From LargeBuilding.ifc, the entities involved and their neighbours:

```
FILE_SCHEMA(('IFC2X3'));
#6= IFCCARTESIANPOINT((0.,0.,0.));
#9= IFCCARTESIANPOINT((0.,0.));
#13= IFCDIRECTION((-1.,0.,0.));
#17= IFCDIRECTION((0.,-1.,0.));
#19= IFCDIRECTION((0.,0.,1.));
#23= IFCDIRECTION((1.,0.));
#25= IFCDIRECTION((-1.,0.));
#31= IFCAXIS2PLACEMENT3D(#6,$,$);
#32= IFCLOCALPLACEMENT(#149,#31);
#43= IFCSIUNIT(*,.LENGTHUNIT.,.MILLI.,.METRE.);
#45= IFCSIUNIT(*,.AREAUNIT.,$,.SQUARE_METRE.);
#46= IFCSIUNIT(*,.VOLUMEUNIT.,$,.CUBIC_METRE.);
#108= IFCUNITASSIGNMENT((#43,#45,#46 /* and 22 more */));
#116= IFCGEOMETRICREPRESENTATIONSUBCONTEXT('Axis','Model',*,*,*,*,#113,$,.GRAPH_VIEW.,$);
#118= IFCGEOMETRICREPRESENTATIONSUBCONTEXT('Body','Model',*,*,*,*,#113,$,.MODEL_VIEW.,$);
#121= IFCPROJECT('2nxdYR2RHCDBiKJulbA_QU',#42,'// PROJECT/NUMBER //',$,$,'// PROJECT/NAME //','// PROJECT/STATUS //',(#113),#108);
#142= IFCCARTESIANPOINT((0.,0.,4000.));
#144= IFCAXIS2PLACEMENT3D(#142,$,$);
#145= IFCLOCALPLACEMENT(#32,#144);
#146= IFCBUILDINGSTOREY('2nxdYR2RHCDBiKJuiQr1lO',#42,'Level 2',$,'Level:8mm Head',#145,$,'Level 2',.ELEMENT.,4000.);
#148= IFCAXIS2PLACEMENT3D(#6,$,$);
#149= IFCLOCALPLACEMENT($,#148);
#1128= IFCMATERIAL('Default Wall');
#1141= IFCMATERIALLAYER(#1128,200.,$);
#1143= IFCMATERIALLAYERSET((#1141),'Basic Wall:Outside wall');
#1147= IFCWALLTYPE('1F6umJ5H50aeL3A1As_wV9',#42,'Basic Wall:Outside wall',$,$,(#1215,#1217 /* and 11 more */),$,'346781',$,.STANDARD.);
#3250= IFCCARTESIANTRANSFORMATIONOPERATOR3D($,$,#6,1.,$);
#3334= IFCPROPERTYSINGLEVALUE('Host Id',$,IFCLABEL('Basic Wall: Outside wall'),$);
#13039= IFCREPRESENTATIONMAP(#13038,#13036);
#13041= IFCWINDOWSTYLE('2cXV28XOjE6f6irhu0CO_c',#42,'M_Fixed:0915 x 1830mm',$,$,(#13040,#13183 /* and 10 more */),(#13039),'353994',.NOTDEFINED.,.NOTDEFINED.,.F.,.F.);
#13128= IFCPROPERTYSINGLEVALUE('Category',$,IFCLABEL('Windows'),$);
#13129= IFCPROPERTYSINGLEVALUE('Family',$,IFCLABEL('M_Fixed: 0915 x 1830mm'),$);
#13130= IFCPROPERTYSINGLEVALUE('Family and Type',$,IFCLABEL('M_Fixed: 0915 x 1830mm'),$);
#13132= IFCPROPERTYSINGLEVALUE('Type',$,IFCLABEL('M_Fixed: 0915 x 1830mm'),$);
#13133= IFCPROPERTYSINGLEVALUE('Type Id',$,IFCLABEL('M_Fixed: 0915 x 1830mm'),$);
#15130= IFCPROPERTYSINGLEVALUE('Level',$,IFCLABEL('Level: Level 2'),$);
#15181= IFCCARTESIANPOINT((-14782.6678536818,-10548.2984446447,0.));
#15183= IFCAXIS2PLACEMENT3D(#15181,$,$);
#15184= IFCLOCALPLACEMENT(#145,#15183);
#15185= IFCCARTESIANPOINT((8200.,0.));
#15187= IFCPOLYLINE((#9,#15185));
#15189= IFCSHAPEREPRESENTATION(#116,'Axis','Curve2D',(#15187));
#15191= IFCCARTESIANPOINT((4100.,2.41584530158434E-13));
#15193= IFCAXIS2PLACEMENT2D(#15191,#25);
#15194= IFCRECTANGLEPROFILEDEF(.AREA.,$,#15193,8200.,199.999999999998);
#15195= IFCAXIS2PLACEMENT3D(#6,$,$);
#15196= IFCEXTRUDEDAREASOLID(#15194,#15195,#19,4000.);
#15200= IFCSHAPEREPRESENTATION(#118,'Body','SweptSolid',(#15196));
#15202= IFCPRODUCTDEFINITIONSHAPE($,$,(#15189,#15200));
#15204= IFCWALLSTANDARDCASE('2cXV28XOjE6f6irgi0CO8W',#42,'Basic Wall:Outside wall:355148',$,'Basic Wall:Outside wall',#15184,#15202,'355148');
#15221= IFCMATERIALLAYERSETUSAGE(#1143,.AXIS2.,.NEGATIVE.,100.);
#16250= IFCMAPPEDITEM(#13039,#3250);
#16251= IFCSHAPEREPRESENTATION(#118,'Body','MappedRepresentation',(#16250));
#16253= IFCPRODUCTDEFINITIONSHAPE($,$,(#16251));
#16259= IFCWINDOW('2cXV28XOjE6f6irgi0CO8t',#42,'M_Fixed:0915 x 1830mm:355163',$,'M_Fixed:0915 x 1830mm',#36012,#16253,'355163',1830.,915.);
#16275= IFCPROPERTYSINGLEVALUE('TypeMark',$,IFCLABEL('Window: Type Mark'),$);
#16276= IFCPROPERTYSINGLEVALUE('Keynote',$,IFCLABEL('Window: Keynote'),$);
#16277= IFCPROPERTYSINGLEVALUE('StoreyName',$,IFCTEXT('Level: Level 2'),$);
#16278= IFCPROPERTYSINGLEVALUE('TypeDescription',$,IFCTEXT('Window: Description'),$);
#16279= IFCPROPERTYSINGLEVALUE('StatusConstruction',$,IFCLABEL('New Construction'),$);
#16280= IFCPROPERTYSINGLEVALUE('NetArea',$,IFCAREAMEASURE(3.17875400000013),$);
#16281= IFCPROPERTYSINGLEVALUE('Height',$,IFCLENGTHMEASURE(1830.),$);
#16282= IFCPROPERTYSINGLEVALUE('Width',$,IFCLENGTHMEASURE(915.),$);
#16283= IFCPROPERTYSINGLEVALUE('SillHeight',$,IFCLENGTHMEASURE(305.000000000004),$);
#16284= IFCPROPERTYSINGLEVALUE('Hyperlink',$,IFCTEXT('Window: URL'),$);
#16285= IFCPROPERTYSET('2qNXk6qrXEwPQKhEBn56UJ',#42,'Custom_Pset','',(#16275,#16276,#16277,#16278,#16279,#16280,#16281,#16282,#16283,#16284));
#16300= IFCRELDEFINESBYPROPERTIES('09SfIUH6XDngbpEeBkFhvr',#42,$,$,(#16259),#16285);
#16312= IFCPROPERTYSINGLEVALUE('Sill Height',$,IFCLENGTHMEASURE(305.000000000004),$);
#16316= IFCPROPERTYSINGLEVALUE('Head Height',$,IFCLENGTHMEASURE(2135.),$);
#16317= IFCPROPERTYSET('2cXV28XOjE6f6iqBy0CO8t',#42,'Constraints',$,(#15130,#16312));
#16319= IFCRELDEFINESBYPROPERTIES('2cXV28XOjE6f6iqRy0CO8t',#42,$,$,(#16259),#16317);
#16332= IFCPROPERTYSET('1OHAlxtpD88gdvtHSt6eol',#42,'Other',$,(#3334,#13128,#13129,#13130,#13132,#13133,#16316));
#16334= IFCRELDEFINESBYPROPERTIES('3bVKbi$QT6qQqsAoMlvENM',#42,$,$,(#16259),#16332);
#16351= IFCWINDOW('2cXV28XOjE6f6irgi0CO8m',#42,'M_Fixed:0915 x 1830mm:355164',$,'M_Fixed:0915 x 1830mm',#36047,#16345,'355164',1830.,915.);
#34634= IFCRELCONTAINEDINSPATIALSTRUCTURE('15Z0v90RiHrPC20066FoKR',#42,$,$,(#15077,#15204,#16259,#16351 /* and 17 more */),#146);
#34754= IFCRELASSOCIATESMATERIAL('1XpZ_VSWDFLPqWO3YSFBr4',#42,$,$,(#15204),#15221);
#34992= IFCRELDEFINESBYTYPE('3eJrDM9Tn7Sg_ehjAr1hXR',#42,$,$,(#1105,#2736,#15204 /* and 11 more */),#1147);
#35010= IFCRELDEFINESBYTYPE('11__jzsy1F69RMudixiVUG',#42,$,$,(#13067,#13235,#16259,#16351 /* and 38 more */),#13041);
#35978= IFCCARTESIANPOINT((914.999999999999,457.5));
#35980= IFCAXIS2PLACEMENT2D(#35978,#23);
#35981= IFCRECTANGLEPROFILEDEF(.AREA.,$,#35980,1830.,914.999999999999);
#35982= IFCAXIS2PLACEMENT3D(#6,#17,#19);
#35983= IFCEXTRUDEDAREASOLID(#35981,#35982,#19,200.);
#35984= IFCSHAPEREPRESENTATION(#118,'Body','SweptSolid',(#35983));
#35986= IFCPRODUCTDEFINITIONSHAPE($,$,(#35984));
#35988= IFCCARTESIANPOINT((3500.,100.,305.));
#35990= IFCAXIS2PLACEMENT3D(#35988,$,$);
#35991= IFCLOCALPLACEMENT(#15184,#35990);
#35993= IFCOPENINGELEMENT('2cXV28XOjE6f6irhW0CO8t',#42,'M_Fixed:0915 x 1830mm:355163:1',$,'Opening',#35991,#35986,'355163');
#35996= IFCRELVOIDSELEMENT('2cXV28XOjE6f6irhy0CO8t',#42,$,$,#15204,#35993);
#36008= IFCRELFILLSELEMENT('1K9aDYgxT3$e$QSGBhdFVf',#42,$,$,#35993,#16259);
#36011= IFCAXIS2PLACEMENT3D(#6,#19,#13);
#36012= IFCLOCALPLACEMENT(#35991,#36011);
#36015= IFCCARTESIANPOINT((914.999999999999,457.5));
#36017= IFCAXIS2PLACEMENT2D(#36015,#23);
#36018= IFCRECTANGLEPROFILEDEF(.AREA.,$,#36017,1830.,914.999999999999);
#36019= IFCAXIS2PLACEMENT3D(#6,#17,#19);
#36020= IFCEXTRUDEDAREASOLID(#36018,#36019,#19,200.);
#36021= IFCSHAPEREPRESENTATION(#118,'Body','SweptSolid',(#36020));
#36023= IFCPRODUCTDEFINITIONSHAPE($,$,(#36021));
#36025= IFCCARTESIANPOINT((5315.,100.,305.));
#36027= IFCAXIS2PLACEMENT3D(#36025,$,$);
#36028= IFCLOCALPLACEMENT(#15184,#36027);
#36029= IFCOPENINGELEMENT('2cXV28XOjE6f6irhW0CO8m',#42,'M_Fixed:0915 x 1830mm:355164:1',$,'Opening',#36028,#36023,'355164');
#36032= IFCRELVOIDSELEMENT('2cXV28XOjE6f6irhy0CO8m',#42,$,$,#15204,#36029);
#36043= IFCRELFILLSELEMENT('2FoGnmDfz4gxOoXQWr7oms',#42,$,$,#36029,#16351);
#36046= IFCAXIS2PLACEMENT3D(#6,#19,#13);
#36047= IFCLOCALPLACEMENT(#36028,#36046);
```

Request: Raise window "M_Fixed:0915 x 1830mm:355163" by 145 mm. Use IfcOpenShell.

```python
import numpy as np
import ifcopenshell
import ifcopenshell.api.geometry
import ifcopenshell.api.pset
import ifcopenshell.util.element
import ifcopenshell.util.placement
import ifcopenshell.util.unit

model = ifcopenshell.open("LargeBuilding.ifc")
unit_scale = ifcopenshell.util.unit.calculate_unit_scale(model)

window = model.by_guid("2cXV28XOjE6f6irgi0CO8t")
opening = window.FillsVoids[0].RelatingOpeningElement
dz = 0.145 / unit_scale

shift = np.array([0.0, 0.0, dz])
# The window is placed relative to its opening, so it follows when the opening moves.
matrix = ifcopenshell.util.placement.get_local_placement(opening.ObjectPlacement)
matrix[:3, 3] += shift
ifcopenshell.api.geometry.edit_object_placement(
    model, product=opening, matrix=matrix, is_si=False, should_transform_children=True
)

# Keep the stored heights in step.
pset = model.by_id(ifcopenshell.util.element.get_pset(window, "Custom_Pset", should_inherit=False)["id"])
ifcopenshell.api.pset.edit_pset(model, pset=pset, properties={
    "SillHeight": model.create_entity("IfcLengthMeasure", ifcopenshell.util.element.get_pset(window, "Constraints", "Sill Height") + dz),
})
pset = model.by_id(ifcopenshell.util.element.get_pset(window, "Constraints", should_inherit=False)["id"])
ifcopenshell.api.pset.edit_pset(model, pset=pset, properties={
    "Sill Height": model.create_entity("IfcLengthMeasure", ifcopenshell.util.element.get_pset(window, "Constraints", "Sill Height") + dz),
})
pset = model.by_id(ifcopenshell.util.element.get_pset(window, "Other", should_inherit=False)["id"])
ifcopenshell.api.pset.edit_pset(model, pset=pset, properties={
    "Head Height": model.create_entity("IfcLengthMeasure", ifcopenshell.util.element.get_pset(window, "Other", "Head Height") + dz),
})

print(f"moved by {dz * unit_scale:+.3f} m")

model.write("LargeBuilding_updated.ifc")
```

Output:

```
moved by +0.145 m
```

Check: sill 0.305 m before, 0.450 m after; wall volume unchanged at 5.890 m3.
